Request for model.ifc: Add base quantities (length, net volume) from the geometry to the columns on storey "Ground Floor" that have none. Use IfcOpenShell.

First a look at what the model holds.

```python
import ifcopenshell
import ifcopenshell.util.element
import ifcopenshell.util.unit

model = ifcopenshell.open("model.ifc")
print(model.schema)
for unit_type in ("LENGTHUNIT", "AREAUNIT", "VOLUMEUNIT"):
    print(unit_type, ifcopenshell.util.unit.calculate_unit_scale(model, unit_type))
storey = next(s for s in model.by_type("IfcBuildingStorey") if s.Name == "Ground Floor")
columns = [e for e in ifcopenshell.util.element.get_decomposition(storey) if e.is_a("IfcColumn")]
for e in sorted(columns, key=lambda e: e.id()):
    print(e.id(), e.is_a(), e.Name, list(ifcopenshell.util.element.get_psets(e, qtos_only=True)), sep=" | ")
```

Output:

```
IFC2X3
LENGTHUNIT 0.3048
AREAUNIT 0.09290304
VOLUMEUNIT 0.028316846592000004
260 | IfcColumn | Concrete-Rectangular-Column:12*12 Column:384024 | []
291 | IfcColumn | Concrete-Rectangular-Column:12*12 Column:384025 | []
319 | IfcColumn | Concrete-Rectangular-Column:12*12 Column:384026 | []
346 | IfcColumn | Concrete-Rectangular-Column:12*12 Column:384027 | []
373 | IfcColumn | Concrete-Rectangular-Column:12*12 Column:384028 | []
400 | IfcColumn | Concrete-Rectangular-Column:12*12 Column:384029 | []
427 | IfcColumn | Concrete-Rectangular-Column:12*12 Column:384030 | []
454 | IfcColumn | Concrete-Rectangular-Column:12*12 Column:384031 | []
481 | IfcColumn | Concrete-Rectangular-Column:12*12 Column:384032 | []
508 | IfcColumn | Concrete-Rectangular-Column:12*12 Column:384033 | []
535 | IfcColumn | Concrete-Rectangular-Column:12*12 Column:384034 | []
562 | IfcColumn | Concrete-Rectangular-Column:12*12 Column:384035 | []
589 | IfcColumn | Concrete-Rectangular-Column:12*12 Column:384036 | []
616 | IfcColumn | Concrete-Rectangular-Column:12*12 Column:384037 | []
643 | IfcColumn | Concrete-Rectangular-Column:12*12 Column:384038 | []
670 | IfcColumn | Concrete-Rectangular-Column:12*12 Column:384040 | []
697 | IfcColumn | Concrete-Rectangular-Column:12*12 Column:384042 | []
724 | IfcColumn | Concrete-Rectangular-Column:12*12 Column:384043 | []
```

```python
import ifcopenshell
import ifcopenshell.api.pset
import ifcopenshell.geom
import ifcopenshell.util.element
import ifcopenshell.util.shape
import ifcopenshell.util.unit

model = ifcopenshell.open("model.ifc")
unit_scale = ifcopenshell.util.unit.calculate_unit_scale(model)
volume_scale = ifcopenshell.util.unit.calculate_unit_scale(model, "VOLUMEUNIT")
settings = ifcopenshell.geom.settings()

storey = next(s for s in model.by_type("IfcBuildingStorey") if s.Name == "Ground Floor")
columns = [e for e in ifcopenshell.util.element.get_decomposition(storey) if e.is_a("IfcColumn")]

for e in sorted(columns, key=lambda e: e.id()):
    if ifcopenshell.util.element.get_psets(e, qtos_only=True, should_inherit=False):
        continue
    # Geometry comes back in metres, in the element's own axes.
    shape = ifcopenshell.geom.create_shape(settings, e)
    values = {
        "Length": ifcopenshell.util.shape.get_z(shape.geometry) / unit_scale,
        "NetVolume": ifcopenshell.util.shape.get_volume(shape.geometry) / volume_scale,
    }
    qto = ifcopenshell.api.pset.add_qto(model, product=e, name="BaseQuantities")
    ifcopenshell.api.pset.edit_qto(model, qto=qto, properties=values)
    print(e.id(), {k: round(v, 3) for k, v in values.items()})

model.write("model_edited.ifc")
```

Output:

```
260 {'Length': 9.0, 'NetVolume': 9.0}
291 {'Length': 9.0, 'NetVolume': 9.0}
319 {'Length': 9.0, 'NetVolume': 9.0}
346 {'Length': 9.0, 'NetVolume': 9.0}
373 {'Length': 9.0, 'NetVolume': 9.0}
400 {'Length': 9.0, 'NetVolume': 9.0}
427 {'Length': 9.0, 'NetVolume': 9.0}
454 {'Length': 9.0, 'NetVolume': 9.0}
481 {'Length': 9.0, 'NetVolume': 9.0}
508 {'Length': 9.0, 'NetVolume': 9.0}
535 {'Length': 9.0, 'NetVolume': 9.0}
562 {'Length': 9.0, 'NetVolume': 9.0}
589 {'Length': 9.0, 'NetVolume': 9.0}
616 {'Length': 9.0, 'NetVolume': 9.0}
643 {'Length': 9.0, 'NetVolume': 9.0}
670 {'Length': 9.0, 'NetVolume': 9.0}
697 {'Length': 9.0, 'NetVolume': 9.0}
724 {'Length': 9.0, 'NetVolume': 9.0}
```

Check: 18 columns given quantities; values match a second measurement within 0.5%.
